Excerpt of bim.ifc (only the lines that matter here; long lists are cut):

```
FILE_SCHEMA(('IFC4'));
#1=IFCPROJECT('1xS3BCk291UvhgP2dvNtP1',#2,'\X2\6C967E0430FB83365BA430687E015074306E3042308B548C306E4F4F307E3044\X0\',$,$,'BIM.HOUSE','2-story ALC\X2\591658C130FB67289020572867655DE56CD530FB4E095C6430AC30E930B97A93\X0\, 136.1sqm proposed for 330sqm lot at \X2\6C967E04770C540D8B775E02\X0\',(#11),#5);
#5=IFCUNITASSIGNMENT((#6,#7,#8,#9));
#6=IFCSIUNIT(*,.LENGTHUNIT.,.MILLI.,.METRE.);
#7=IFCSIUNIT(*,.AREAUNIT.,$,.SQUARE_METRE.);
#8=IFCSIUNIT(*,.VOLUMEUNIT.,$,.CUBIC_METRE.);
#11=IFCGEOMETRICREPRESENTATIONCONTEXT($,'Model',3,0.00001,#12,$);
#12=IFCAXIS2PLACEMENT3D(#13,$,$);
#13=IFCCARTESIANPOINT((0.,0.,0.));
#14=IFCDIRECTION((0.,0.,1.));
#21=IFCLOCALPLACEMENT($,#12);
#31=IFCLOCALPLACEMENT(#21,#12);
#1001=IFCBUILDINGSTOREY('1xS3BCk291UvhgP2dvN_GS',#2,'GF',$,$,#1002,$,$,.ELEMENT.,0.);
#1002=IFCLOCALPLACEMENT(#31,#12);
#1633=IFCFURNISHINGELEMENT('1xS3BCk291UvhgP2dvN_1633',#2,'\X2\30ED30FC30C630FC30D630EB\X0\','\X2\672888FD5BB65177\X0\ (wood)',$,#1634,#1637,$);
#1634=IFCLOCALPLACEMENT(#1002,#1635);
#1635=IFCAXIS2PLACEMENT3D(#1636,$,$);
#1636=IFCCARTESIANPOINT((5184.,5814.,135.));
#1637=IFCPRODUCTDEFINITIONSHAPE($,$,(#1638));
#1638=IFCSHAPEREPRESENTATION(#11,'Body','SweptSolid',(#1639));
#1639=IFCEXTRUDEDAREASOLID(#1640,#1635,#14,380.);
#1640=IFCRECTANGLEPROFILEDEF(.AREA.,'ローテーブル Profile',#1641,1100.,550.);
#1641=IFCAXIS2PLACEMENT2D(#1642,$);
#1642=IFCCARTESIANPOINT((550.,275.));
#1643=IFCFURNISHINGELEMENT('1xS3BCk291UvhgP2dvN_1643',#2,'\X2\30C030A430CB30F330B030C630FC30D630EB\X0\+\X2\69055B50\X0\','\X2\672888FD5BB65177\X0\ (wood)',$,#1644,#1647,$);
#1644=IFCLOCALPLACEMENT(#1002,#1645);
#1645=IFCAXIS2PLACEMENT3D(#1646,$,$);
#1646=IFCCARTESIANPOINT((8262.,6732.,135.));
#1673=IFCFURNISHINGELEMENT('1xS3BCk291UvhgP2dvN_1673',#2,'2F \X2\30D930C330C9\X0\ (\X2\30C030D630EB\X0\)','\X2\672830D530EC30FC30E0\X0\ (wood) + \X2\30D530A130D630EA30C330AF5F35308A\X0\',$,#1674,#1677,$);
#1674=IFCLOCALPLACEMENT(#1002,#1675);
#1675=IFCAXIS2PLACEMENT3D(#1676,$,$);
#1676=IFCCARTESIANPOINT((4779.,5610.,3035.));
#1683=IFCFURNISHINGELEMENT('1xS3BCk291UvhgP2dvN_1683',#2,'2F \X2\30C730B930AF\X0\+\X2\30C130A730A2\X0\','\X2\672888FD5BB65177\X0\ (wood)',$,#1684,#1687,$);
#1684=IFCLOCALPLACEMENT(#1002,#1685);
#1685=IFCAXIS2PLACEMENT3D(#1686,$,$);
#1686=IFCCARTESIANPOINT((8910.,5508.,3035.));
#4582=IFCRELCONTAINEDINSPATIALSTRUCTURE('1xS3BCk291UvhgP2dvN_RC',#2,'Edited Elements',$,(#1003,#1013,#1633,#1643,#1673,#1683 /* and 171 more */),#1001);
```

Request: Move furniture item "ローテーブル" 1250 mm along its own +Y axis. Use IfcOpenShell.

```python
import ifcopenshell
import ifcopenshell.api.geometry
import ifcopenshell.util.placement

model = ifcopenshell.open("bim.ifc")

item = model.by_guid("1xS3BCk291UvhgP2dvN_1633")
matrix = ifcopenshell.util.placement.get_local_placement(item.ObjectPlacement)
matrix[:3, 3] += matrix[:3, 1] * 1250.0
ifcopenshell.api.geometry.edit_object_placement(model, product=item, matrix=matrix, is_si=False)

print(ifcopenshell.util.placement.get_local_placement(item.ObjectPlacement).round(3) + 0.0)

model.write("bim_v2.ifc")
```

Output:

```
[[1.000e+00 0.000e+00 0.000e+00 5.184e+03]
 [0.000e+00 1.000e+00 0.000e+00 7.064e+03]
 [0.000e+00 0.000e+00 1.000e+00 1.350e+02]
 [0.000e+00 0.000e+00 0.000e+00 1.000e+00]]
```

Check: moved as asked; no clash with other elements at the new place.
